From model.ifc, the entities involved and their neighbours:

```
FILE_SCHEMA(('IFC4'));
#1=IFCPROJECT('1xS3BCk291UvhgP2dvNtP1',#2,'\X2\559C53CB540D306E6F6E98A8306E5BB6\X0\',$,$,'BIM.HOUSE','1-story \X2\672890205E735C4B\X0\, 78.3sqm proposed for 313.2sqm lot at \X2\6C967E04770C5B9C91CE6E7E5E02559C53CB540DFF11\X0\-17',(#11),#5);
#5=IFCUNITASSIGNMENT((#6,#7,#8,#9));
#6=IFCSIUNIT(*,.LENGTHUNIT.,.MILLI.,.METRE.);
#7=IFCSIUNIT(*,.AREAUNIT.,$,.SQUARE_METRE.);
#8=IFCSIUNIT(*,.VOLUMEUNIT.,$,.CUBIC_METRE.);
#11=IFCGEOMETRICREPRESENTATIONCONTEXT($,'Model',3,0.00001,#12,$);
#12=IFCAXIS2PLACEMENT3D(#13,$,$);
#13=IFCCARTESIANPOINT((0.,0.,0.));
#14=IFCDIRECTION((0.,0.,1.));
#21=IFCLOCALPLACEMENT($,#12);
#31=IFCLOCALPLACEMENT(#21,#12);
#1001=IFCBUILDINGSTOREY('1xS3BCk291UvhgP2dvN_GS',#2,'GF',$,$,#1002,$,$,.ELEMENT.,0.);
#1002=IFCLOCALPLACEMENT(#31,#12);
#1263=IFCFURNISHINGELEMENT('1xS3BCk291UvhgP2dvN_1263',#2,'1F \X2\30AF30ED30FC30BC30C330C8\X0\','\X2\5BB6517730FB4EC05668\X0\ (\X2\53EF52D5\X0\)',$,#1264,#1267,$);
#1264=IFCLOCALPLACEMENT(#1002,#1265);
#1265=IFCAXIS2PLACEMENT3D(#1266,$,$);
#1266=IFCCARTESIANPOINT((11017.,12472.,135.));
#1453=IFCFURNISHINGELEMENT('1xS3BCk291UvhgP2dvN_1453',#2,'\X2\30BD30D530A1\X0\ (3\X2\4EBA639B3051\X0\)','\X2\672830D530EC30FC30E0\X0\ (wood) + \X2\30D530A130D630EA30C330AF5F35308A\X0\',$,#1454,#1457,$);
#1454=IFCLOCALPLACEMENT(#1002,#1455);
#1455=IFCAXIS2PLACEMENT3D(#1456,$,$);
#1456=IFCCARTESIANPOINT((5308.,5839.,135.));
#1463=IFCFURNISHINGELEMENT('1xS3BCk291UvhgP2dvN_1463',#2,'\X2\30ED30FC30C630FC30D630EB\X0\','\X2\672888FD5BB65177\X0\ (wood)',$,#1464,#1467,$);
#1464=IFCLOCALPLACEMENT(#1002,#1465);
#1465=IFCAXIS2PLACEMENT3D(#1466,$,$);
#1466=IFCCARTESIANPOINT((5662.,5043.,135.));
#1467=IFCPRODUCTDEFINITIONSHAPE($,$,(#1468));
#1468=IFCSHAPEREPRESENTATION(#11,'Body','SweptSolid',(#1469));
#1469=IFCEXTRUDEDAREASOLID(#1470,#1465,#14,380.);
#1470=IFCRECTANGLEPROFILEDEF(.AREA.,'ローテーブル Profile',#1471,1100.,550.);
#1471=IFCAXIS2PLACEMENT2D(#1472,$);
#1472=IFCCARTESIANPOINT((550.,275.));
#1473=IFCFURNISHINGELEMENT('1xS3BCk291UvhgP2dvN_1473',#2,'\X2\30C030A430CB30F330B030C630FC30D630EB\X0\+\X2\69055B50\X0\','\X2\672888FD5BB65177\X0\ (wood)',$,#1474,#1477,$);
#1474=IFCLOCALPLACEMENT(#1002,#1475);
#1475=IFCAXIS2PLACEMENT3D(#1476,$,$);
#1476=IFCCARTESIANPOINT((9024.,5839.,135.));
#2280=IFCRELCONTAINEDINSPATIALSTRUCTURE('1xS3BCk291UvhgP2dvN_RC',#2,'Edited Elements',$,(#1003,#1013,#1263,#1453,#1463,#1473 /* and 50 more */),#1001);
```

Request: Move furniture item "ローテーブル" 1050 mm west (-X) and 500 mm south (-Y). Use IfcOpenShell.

```python
import ifcopenshell
import ifcopenshell.api.geometry
import ifcopenshell.util.placement
import ifcopenshell.util.unit

model = ifcopenshell.open("model.ifc")
unit_scale = ifcopenshell.util.unit.calculate_unit_scale(model)

item = model.by_id(1463)
matrix = ifcopenshell.util.placement.get_local_placement(item.ObjectPlacement)
matrix[0, 3] -= 1.05 / unit_scale
matrix[1, 3] -= 0.5 / unit_scale
ifcopenshell.api.geometry.edit_object_placement(model, product=item, matrix=matrix, is_si=False)

print(ifcopenshell.util.placement.get_local_placement(item.ObjectPlacement).round(3) + 0.0)

model.write("model_edited.ifc")
```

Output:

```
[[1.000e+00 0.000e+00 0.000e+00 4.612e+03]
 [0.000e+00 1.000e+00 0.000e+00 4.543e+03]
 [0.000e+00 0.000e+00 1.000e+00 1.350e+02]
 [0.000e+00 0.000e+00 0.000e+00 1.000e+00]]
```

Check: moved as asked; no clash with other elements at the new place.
